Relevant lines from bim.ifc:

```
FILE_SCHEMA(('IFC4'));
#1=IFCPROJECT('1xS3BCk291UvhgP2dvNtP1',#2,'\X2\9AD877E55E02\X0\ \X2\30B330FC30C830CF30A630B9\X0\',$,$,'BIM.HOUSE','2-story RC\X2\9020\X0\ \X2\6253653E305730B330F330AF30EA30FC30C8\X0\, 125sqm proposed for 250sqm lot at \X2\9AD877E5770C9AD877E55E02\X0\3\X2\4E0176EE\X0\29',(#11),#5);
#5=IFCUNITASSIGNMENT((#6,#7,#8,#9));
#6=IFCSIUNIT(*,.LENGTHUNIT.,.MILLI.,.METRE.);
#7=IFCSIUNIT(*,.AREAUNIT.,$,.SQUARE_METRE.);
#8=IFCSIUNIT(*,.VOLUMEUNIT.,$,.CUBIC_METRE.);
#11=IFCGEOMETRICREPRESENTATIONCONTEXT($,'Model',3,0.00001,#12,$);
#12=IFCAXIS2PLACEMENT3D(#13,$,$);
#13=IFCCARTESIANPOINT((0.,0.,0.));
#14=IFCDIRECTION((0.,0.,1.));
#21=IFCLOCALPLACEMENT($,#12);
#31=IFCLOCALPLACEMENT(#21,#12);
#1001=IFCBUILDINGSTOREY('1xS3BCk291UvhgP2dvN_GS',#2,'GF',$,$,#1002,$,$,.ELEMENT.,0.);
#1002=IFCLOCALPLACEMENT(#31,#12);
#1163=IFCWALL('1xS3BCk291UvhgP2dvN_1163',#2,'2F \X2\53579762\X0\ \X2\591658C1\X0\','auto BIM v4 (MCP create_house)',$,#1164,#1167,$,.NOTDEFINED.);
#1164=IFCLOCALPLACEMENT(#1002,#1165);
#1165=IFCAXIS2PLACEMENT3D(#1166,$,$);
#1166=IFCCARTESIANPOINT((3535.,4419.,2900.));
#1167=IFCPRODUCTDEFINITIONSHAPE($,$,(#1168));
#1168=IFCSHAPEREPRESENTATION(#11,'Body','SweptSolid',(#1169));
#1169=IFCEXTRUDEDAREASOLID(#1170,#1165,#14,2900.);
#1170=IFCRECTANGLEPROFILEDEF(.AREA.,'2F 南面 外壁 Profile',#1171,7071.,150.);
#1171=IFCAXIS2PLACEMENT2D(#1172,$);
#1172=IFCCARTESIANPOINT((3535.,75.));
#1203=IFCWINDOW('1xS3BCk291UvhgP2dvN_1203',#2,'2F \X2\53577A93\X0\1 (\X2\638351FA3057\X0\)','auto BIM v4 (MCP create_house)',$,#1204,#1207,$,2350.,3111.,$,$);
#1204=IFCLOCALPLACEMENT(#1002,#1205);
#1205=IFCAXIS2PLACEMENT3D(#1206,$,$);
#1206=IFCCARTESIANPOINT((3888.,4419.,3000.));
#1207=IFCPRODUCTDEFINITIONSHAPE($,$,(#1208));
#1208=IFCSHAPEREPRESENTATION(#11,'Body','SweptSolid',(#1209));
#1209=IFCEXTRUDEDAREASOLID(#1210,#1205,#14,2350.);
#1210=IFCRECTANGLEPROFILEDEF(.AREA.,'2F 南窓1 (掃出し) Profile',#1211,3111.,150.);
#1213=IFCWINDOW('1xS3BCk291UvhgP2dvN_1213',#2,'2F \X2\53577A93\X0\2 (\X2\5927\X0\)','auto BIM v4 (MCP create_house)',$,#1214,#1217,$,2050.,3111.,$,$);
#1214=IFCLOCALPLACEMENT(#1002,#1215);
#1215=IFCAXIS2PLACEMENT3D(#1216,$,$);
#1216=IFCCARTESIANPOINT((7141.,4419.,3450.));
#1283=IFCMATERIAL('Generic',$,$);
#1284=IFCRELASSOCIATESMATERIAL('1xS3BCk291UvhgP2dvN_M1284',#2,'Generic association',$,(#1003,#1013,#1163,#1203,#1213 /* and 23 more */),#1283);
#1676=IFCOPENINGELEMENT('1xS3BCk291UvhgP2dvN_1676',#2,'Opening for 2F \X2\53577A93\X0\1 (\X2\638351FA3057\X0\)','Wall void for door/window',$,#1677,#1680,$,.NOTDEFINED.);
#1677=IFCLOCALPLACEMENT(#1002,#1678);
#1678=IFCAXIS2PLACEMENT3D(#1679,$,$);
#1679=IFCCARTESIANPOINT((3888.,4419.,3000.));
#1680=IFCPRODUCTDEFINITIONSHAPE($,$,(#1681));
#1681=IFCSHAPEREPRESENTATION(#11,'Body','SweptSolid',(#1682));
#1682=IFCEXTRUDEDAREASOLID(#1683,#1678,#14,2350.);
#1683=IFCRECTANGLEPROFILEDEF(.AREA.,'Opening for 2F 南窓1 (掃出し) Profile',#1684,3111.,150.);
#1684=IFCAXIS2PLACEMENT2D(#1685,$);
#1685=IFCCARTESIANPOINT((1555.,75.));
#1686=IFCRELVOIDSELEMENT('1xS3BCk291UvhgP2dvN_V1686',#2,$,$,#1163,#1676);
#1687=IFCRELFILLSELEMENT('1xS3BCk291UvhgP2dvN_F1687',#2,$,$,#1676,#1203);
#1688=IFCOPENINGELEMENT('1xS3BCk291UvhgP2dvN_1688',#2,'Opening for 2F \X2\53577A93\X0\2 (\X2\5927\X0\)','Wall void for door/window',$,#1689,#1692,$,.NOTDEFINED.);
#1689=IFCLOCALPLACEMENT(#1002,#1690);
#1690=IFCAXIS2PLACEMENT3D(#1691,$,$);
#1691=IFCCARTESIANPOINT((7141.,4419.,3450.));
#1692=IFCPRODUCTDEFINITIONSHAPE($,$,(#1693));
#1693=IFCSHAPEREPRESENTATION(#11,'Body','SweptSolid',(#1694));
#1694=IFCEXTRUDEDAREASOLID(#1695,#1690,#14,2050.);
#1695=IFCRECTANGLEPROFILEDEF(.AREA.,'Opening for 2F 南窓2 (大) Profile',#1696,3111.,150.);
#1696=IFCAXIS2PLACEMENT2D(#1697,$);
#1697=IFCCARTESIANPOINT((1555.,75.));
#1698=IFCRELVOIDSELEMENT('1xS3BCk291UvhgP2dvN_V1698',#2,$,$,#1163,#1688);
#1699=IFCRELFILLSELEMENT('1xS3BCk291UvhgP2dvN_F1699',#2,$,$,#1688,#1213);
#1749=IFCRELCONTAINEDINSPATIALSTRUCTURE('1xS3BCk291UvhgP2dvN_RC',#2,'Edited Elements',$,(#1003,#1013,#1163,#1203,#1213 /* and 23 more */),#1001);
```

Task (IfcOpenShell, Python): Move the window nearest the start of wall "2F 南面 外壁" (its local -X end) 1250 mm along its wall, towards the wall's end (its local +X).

```python
import ifcopenshell
import ifcopenshell.api.geometry
import ifcopenshell.util.placement
import ifcopenshell.util.unit

model = ifcopenshell.open("bim.ifc")
unit_scale = ifcopenshell.util.unit.calculate_unit_scale(model)

window = model.by_guid("1xS3BCk291UvhgP2dvN_1203")
opening = window.FillsVoids[0].RelatingOpeningElement
wall = opening.VoidsElements[0].RelatingBuildingElement

wall_matrix = ifcopenshell.util.placement.get_local_placement(wall.ObjectPlacement)
shift = wall_matrix[:3, 0] * 1.25 / unit_scale
before = ifcopenshell.util.placement.get_local_placement(window.ObjectPlacement)[:3, 3].copy()

# The window is not placed relative to its opening, so move both.
for product in (opening, window):
    matrix = ifcopenshell.util.placement.get_local_placement(product.ObjectPlacement)
    matrix[:3, 3] += shift
    ifcopenshell.api.geometry.edit_object_placement(model, product=product, matrix=matrix, is_si=False)

after = ifcopenshell.util.placement.get_local_placement(window.ObjectPlacement)[:3, 3]
print("window moved by", (after - before).round(3) + 0.0)

model.write("bim_v2.ifc")
```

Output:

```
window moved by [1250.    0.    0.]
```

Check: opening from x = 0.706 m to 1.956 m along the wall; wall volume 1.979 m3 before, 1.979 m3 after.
